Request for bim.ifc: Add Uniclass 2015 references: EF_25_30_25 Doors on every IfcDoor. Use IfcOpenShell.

First a look at what the model holds.

```python
import ifcopenshell

model = ifcopenshell.open("bim.ifc")
print(model.schema)
print("classifications:", [c.Name for c in model.by_type("IfcClassification")])
for ifc_class in ("IfcDoor", "IfcRoof", "IfcStair", "IfcWall", "IfcWindow"):
    print(ifc_class, len(model.by_type(ifc_class)))
```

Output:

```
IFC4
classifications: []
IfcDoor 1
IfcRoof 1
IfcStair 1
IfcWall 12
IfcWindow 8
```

```python
import ifcopenshell
import ifcopenshell.api.classification

model = ifcopenshell.open("bim.ifc")

system = ifcopenshell.api.classification.add_classification(model, classification="Uniclass 2015")

codes = {
    "IfcDoor": ("EF_25_30_25", "Doors"),
}
for ifc_class, (code, name) in codes.items():
    products = model.by_type(ifc_class)
    ifcopenshell.api.classification.add_reference(
        model, products=products, classification=system, identification=code, name=name
    )
    print(code, len(products))

model.write("bim_updated.ifc")
```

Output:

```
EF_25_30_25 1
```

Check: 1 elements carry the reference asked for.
